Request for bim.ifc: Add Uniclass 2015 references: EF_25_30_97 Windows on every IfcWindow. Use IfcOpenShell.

First a look at what the model holds.

```python
import ifcopenshell

model = ifcopenshell.open("bim.ifc")
print(model.schema)
print("classifications:", [c.Name for c in model.by_type("IfcClassification")])
for ifc_class in ("IfcDoor", "IfcRoof", "IfcStair", "IfcWall", "IfcWindow"):
    print(ifc_class, len(model.by_type(ifc_class)))
```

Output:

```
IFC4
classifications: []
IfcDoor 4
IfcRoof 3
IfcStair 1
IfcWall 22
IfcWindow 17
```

```python
import ifcopenshell
import ifcopenshell.api.classification

model = ifcopenshell.open("bim.ifc")

system = ifcopenshell.api.classification.add_classification(model, classification="Uniclass 2015")

codes = {
    "IfcWindow": ("EF_25_30_97", "Windows"),
}
for ifc_class, (code, name) in codes.items():
    products = model.by_type(ifc_class)
    ifcopenshell.api.classification.add_reference(
        model, products=products, classification=system, identification=code, name=name
    )
    print(code, len(products))

model.write("bim_updated.ifc")
```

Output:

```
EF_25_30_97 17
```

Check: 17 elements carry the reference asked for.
